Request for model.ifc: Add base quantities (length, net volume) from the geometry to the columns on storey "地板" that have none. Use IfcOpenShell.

First a look at what the model holds.

```python
import ifcopenshell
import ifcopenshell.util.element
import ifcopenshell.util.unit

model = ifcopenshell.open("model.ifc")
print(model.schema)
for unit_type in ("LENGTHUNIT", "AREAUNIT", "VOLUMEUNIT"):
    print(unit_type, ifcopenshell.util.unit.calculate_unit_scale(model, unit_type))
storey = next(s for s in model.by_type("IfcBuildingStorey") if s.Name == "地板")
columns = [e for e in ifcopenshell.util.element.get_decomposition(storey) if e.is_a("IfcColumn")]
for e in sorted(columns, key=lambda e: e.id()):
    print(e.id(), e.is_a(), e.Name, list(ifcopenshell.util.element.get_psets(e, qtos_only=True)), sep=" | ")
```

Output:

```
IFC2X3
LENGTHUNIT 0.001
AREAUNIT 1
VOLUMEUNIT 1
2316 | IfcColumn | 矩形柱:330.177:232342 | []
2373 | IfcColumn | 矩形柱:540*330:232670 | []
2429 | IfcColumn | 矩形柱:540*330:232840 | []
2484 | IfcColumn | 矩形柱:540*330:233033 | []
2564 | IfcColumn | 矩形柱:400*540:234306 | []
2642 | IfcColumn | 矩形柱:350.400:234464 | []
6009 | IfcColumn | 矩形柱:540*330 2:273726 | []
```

```python
import ifcopenshell
import ifcopenshell.api.pset
import ifcopenshell.geom
import ifcopenshell.util.element
import ifcopenshell.util.shape
import ifcopenshell.util.unit

model = ifcopenshell.open("model.ifc")
unit_scale = ifcopenshell.util.unit.calculate_unit_scale(model)
volume_scale = ifcopenshell.util.unit.calculate_unit_scale(model, "VOLUMEUNIT")
settings = ifcopenshell.geom.settings()

storey = next(s for s in model.by_type("IfcBuildingStorey") if s.Name == "地板")
columns = [e for e in ifcopenshell.util.element.get_decomposition(storey) if e.is_a("IfcColumn")]

for e in sorted(columns, key=lambda e: e.id()):
    if ifcopenshell.util.element.get_psets(e, qtos_only=True, should_inherit=False):
        continue
    # Geometry comes back in metres, in the element's own axes.
    shape = ifcopenshell.geom.create_shape(settings, e)
    values = {
        "Length": ifcopenshell.util.shape.get_z(shape.geometry) / unit_scale,
        "NetVolume": ifcopenshell.util.shape.get_volume(shape.geometry) / volume_scale,
    }
    qto = ifcopenshell.api.pset.add_qto(model, product=e, name="BaseQuantities")
    ifcopenshell.api.pset.edit_qto(model, qto=qto, properties=values)
    print(e.id(), {k: round(v, 3) for k, v in values.items()})

model.write("model-out.ifc")
```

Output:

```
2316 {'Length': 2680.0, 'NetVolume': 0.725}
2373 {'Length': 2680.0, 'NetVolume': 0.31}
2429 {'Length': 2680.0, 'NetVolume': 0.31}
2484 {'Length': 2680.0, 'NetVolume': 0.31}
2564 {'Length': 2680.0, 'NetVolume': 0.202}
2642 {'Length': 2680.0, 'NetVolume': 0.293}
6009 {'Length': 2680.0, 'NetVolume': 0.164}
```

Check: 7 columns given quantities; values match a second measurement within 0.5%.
